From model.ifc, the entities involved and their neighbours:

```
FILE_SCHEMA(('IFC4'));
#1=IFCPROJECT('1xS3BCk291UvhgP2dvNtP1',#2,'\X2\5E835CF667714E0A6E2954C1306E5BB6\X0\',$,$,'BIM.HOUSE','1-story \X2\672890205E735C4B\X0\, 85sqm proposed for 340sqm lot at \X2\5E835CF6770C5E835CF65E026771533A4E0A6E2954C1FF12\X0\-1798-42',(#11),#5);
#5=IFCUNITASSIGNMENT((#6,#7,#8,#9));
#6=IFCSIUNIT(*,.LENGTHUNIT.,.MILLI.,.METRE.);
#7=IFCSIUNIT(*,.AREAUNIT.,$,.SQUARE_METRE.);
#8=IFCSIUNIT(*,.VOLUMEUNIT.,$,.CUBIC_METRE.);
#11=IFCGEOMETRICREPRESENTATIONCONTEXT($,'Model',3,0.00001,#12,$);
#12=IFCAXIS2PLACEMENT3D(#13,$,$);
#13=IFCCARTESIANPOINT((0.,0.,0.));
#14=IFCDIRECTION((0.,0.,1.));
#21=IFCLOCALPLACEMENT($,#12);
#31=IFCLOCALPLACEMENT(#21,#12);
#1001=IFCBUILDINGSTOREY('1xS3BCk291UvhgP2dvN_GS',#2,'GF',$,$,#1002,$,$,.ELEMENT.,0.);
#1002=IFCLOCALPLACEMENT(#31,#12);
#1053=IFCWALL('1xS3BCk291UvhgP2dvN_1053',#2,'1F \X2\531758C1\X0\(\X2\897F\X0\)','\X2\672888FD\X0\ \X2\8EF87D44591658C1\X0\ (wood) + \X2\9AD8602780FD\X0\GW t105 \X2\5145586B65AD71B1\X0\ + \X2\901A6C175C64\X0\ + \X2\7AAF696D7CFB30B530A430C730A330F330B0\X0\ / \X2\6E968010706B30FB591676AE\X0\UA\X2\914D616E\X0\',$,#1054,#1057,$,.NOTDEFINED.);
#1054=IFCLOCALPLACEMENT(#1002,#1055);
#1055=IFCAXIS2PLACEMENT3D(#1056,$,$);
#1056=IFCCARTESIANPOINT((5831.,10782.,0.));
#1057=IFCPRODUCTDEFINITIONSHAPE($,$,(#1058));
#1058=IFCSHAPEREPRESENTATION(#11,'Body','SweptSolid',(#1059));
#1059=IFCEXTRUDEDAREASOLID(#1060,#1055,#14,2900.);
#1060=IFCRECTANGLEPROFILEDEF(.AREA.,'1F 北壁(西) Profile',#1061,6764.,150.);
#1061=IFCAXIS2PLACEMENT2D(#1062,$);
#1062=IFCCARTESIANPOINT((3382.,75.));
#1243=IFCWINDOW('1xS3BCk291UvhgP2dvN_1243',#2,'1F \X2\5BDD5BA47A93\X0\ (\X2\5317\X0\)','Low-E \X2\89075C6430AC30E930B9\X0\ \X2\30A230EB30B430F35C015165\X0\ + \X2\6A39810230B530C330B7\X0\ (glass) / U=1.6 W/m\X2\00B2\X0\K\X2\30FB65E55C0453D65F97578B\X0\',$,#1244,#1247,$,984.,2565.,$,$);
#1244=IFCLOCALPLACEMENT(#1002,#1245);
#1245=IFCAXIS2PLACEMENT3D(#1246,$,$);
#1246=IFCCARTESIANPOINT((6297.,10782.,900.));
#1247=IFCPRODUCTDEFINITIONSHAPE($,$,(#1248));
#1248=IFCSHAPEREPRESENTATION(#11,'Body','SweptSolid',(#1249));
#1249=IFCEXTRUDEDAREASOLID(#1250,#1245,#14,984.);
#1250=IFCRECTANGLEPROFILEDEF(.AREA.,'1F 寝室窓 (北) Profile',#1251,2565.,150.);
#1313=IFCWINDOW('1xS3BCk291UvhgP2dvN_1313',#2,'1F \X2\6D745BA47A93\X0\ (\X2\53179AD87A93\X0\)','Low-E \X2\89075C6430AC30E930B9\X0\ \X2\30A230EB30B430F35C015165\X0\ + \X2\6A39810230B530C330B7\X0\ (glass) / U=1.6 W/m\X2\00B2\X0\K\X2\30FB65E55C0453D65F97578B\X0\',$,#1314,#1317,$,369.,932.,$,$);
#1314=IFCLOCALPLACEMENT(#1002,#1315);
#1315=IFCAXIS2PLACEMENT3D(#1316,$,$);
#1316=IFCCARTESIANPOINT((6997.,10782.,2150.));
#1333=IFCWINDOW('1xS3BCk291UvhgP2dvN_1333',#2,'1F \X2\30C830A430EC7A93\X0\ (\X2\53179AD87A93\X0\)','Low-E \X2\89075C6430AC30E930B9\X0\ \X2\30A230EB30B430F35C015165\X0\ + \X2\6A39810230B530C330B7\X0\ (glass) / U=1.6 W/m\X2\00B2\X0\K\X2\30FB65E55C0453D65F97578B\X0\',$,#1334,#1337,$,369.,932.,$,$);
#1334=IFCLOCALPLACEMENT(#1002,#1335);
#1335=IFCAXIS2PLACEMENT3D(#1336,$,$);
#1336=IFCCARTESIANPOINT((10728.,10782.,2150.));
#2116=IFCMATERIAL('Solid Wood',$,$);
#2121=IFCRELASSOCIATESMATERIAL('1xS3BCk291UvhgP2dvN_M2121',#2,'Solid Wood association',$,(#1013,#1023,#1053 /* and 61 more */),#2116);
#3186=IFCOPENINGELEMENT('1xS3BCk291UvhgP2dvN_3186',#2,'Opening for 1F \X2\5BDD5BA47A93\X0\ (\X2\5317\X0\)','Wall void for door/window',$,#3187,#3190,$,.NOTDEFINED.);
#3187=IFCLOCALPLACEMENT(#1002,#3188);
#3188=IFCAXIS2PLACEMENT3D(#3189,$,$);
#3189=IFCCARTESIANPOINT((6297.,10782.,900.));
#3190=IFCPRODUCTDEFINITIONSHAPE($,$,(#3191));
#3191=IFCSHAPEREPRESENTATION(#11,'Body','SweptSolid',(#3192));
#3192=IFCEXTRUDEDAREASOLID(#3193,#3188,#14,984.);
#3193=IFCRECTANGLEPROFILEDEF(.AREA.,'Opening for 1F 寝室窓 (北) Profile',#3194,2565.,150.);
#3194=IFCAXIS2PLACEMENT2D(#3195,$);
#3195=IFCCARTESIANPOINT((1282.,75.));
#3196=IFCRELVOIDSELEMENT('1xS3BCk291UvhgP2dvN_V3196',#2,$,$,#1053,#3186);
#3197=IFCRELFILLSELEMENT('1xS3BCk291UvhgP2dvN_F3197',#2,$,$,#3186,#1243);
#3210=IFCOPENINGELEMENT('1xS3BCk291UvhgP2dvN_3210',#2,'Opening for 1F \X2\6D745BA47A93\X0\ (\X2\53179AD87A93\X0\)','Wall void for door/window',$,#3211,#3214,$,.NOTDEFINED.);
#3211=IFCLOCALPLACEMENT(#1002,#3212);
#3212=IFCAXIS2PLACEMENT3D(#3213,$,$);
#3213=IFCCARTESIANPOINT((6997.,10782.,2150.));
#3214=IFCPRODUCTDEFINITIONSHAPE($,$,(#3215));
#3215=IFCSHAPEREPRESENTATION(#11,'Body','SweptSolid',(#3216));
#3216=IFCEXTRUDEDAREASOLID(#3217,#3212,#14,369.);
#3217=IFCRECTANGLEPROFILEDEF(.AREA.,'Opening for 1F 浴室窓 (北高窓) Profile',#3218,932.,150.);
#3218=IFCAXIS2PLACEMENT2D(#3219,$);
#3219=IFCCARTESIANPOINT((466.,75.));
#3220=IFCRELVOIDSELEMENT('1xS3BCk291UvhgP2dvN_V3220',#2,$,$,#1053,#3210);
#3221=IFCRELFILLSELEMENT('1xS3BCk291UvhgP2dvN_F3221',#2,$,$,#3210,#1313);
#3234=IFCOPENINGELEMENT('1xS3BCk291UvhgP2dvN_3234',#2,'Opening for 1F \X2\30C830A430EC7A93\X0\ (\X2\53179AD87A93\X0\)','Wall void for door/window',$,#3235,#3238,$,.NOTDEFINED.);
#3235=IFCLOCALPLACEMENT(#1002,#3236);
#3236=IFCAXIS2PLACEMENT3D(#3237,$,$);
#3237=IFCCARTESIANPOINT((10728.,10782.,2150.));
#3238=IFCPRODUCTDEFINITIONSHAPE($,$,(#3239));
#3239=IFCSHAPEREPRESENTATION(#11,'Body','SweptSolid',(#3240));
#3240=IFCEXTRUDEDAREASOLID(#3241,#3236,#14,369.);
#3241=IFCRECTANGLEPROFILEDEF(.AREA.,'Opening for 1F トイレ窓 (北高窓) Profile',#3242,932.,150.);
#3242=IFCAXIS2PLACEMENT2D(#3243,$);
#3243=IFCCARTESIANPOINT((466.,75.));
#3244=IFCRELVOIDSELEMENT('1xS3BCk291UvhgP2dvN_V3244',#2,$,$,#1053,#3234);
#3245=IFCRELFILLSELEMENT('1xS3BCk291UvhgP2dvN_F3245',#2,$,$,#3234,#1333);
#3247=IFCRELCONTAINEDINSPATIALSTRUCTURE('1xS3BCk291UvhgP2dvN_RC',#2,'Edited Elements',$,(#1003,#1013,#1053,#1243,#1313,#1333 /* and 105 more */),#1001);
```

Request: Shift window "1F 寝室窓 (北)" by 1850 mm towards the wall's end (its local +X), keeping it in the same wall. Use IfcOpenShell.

```python
import ifcopenshell
import ifcopenshell.api.geometry
import ifcopenshell.util.placement

model = ifcopenshell.open("model.ifc")

window = model.by_guid("1xS3BCk291UvhgP2dvN_1243")
opening = window.FillsVoids[0].RelatingOpeningElement
wall = opening.VoidsElements[0].RelatingBuildingElement

wall_matrix = ifcopenshell.util.placement.get_local_placement(wall.ObjectPlacement)
shift = wall_matrix[:3, 0] * 1850.0
before = ifcopenshell.util.placement.get_local_placement(window.ObjectPlacement)[:3, 3].copy()

# The window is not placed relative to its opening, so move both.
for product in (opening, window):
    matrix = ifcopenshell.util.placement.get_local_placement(product.ObjectPlacement)
    matrix[:3, 3] += shift
    ifcopenshell.api.geometry.edit_object_placement(model, product=product, matrix=matrix, is_si=False)

after = ifcopenshell.util.placement.get_local_placement(window.ObjectPlacement)[:3, 3]
print("window moved by", (after - before).round(3) + 0.0)

model.write("model_edited.ifc")
```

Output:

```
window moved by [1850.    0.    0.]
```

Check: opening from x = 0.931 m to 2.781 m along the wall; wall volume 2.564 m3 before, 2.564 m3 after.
